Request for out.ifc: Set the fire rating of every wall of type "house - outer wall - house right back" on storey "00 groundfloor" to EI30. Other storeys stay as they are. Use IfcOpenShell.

First a look at what the model holds.

```python
import ifcopenshell
import ifcopenshell.util.element

model = ifcopenshell.open("out.ifc")
print(model.schema)
storey = next(s for s in model.by_type("IfcBuildingStorey") if s.Name == "00 groundfloor")
walls = [e for e in ifcopenshell.util.element.get_decomposition(storey) if e.is_a("IfcWall")]
seen = {}
for e in walls:
    element_type = ifcopenshell.util.element.get_type(e)
    key = (element_type.Name if element_type != e and element_type else None, ifcopenshell.util.element.get_pset(e, "Pset_WallCommon", "FireRating"))
    seen[key] = seen.get(key, 0) + 1
for (name, value), count in sorted(seen.items(), key=str):
    print(count, "x", name, "|", value)
```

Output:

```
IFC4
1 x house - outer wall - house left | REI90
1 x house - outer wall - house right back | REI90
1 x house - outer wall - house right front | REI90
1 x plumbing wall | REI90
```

```python
import ifcopenshell
import ifcopenshell.api.pset
import ifcopenshell.util.element

model = ifcopenshell.open("out.ifc")

storey = next(s for s in model.by_type("IfcBuildingStorey") if s.Name == "00 groundfloor")
walls = [e for e in ifcopenshell.util.element.get_decomposition(storey) if e.is_a("IfcWall")]

count = 0
for e in walls:
    element_type = ifcopenshell.util.element.get_type(e)
    if element_type in (None, e) or element_type.Name != "house - outer wall - house right back":
        continue
    # add_pset returns the element's existing set when there is one.
    pset = ifcopenshell.api.pset.add_pset(model, product=e, name="Pset_WallCommon")
    ifcopenshell.api.pset.edit_pset(model, pset=pset, properties={"FireRating": "EI30"})
    count += 1

print(count, "walls updated")

model.write("out_edited.ifc")
```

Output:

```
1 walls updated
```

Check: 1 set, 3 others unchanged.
